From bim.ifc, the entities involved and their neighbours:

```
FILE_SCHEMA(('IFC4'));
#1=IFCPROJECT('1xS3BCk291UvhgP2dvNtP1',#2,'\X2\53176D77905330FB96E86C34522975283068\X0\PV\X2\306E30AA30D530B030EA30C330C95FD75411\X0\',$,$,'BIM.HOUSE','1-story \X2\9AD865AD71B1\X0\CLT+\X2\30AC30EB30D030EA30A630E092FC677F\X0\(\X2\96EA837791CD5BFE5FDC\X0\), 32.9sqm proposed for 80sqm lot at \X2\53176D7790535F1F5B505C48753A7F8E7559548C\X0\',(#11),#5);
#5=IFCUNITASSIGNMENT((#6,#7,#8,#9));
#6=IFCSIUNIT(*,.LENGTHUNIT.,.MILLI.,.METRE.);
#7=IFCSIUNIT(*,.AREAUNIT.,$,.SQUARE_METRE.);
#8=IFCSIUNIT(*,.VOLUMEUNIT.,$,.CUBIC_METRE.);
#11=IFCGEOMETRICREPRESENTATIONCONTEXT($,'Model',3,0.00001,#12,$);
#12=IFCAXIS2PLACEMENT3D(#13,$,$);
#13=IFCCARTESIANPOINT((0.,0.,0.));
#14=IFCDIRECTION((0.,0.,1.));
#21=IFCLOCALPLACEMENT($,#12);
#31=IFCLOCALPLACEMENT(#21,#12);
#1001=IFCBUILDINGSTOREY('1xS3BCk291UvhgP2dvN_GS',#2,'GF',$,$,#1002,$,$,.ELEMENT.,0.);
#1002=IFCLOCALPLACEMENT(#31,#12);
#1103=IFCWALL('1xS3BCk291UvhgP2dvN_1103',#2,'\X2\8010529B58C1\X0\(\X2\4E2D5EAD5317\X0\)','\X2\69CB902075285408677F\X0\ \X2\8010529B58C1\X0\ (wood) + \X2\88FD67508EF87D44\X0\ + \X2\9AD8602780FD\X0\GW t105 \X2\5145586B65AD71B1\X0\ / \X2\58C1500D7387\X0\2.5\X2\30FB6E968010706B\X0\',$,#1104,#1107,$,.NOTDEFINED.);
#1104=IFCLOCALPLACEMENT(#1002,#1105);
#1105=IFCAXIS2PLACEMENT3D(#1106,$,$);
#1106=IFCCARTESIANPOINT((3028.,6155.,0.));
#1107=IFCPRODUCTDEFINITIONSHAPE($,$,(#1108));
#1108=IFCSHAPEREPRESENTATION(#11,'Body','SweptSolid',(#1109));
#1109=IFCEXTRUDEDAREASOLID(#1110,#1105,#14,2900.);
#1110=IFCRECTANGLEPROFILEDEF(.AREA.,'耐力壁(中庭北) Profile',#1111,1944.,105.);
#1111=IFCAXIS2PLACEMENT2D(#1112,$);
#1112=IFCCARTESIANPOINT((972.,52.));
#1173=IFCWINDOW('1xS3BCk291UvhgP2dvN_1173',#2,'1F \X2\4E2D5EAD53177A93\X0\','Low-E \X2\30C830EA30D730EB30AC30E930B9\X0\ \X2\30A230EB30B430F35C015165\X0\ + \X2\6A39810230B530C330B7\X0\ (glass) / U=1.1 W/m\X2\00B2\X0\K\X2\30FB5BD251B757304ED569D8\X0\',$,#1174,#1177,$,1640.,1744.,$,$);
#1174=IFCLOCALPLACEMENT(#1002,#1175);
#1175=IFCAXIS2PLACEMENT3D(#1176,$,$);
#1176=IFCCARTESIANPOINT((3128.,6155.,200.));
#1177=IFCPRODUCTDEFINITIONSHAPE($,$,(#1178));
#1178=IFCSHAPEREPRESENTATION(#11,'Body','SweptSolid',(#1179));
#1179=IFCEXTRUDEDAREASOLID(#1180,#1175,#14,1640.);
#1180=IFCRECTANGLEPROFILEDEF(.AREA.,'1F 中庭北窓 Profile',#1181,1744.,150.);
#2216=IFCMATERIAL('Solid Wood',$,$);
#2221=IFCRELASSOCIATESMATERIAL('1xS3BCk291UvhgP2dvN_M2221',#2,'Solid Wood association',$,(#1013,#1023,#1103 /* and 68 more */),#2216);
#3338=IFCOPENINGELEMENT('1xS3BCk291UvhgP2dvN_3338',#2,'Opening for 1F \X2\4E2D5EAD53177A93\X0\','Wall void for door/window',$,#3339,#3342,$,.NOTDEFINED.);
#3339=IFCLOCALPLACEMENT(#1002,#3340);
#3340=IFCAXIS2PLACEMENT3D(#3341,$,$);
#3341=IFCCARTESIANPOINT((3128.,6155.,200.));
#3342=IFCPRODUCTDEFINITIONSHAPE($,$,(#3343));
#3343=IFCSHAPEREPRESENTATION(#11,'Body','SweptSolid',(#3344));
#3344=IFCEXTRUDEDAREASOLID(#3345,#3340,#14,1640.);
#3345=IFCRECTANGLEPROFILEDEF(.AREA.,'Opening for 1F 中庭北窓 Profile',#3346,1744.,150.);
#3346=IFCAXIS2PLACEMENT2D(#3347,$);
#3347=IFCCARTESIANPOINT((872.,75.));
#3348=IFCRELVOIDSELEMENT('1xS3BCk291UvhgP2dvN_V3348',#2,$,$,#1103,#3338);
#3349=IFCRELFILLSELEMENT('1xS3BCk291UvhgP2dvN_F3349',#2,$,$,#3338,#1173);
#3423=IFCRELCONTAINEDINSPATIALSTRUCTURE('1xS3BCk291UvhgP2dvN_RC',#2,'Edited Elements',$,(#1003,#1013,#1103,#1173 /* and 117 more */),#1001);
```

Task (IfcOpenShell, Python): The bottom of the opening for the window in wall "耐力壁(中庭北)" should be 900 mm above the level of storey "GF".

```python
import numpy as np
import ifcopenshell
import ifcopenshell.api.geometry
import ifcopenshell.geom
import ifcopenshell.util.element
import ifcopenshell.util.placement
import ifcopenshell.util.shape
import ifcopenshell.util.unit

model = ifcopenshell.open("bim.ifc")
unit_scale = ifcopenshell.util.unit.calculate_unit_scale(model)

window = model.by_id(1173)
opening = window.FillsVoids[0].RelatingOpeningElement
storey = ifcopenshell.util.element.get_container(window, ifc_class="IfcBuildingStorey")
level = ifcopenshell.util.placement.get_local_placement(storey.ObjectPlacement)[2, 3]

# The opening's origin need not be at the sill, so measure its lowest point.
shape = ifcopenshell.geom.create_shape(ifcopenshell.geom.settings(), opening)
bottom = ifcopenshell.util.shape.get_shape_bottom_elevation(shape, shape.geometry) / unit_scale
dz = level + 0.9 / unit_scale - bottom

shift = np.array([0.0, 0.0, dz])
# The window is not placed relative to its opening, so move both.
for product in (opening, window):
    matrix = ifcopenshell.util.placement.get_local_placement(product.ObjectPlacement)
    matrix[:3, 3] += shift
    ifcopenshell.api.geometry.edit_object_placement(model, product=product, matrix=matrix, is_si=False)

print(f"moved by {dz * unit_scale:+.3f} m")

model.write("bim_v2.ifc")
```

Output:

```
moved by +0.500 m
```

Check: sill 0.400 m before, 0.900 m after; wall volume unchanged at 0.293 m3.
